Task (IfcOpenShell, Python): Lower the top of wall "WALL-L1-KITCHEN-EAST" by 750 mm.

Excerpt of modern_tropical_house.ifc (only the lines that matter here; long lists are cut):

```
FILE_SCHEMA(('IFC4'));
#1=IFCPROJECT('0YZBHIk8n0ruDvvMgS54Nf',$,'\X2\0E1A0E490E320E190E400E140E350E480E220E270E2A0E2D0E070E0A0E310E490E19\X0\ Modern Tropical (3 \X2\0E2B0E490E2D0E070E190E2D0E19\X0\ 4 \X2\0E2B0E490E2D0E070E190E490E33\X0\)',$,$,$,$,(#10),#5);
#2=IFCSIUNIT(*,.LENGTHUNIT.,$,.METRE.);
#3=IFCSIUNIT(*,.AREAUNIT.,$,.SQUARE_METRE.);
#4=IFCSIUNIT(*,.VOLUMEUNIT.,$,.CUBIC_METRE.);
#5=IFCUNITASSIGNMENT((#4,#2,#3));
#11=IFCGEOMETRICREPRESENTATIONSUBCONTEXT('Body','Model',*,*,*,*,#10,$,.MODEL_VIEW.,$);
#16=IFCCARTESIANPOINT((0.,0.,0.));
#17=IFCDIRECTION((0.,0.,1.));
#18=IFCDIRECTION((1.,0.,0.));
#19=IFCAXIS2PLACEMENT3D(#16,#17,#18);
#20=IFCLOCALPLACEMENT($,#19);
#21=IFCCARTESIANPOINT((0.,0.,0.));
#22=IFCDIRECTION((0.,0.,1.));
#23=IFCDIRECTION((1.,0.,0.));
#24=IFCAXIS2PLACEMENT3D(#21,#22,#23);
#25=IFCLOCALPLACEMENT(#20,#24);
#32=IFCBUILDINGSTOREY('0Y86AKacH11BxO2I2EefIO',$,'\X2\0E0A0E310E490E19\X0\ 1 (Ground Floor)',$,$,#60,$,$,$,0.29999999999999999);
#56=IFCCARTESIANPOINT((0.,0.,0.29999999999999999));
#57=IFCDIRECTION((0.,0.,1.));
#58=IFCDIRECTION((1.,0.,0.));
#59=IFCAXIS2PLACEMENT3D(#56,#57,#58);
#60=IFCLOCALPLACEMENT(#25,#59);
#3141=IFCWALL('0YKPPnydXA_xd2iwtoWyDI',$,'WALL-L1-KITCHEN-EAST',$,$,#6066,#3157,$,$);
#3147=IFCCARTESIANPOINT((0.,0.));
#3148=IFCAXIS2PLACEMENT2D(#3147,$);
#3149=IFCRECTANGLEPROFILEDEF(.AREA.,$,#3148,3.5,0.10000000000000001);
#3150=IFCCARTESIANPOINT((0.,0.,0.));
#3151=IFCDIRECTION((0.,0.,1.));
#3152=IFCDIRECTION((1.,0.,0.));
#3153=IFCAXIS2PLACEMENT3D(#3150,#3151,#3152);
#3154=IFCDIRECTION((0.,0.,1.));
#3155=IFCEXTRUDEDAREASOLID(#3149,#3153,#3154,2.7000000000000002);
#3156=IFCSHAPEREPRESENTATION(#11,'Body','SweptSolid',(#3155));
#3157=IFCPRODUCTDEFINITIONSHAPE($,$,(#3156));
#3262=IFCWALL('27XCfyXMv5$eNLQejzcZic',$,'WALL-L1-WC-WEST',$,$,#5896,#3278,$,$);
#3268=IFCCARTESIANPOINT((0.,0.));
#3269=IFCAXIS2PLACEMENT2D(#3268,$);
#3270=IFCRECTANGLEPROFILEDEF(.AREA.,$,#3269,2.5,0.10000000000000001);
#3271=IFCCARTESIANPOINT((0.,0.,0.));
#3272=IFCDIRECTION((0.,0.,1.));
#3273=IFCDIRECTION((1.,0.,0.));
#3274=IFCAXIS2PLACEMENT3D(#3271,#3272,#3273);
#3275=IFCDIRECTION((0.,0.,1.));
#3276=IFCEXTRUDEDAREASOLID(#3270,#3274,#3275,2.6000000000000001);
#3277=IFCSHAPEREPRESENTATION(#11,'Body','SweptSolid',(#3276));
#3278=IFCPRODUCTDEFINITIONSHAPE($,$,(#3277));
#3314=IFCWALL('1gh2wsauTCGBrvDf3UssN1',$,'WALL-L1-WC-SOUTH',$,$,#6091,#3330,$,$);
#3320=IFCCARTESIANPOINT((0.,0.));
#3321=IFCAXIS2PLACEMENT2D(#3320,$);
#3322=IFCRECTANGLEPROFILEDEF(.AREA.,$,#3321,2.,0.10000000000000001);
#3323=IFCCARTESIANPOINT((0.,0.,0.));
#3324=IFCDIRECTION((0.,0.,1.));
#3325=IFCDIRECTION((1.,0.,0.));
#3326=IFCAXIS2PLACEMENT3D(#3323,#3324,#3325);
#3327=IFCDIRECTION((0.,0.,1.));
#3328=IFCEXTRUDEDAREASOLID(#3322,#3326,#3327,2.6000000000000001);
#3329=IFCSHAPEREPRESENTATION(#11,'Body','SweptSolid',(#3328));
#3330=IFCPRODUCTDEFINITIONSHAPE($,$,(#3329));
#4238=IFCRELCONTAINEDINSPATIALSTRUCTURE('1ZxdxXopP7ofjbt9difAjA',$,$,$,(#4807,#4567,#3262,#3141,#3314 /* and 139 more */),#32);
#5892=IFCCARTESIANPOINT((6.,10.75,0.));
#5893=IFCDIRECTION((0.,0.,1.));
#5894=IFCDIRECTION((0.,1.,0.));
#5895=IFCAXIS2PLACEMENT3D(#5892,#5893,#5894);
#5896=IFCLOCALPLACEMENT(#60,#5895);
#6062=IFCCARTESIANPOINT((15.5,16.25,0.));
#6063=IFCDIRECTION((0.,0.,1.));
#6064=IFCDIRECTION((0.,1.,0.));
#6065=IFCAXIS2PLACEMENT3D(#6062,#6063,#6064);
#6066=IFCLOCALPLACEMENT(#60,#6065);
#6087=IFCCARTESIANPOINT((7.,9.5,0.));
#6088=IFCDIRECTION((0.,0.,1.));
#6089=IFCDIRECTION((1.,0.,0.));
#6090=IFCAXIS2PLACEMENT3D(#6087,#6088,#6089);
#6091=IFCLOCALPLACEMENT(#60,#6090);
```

```python
import ifcopenshell
import ifcopenshell.geom
import ifcopenshell.util.representation
import ifcopenshell.util.shape

model = ifcopenshell.open("modern_tropical_house.ifc")
settings = ifcopenshell.geom.settings()


def volume(element):
    """Net volume in cubic metres, openings subtracted."""
    shape = ifcopenshell.geom.create_shape(settings, element)
    return ifcopenshell.util.shape.get_volume(shape.geometry)


wall = model.by_id(3141)
before = volume(wall)

body = ifcopenshell.util.representation.get_representation(wall, "Model", "Body")
solid = body.Items[0]
old_height = solid.Depth
solid.Depth -= 0.75
after = volume(wall)

print(f"height {old_height:g} -> {solid.Depth:g}, volume {before:.3f} -> {after:.3f} m3")

model.write("modern_tropical_house_v2.ifc")
```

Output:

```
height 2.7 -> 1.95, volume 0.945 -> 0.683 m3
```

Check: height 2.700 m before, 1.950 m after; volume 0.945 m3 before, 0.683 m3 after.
